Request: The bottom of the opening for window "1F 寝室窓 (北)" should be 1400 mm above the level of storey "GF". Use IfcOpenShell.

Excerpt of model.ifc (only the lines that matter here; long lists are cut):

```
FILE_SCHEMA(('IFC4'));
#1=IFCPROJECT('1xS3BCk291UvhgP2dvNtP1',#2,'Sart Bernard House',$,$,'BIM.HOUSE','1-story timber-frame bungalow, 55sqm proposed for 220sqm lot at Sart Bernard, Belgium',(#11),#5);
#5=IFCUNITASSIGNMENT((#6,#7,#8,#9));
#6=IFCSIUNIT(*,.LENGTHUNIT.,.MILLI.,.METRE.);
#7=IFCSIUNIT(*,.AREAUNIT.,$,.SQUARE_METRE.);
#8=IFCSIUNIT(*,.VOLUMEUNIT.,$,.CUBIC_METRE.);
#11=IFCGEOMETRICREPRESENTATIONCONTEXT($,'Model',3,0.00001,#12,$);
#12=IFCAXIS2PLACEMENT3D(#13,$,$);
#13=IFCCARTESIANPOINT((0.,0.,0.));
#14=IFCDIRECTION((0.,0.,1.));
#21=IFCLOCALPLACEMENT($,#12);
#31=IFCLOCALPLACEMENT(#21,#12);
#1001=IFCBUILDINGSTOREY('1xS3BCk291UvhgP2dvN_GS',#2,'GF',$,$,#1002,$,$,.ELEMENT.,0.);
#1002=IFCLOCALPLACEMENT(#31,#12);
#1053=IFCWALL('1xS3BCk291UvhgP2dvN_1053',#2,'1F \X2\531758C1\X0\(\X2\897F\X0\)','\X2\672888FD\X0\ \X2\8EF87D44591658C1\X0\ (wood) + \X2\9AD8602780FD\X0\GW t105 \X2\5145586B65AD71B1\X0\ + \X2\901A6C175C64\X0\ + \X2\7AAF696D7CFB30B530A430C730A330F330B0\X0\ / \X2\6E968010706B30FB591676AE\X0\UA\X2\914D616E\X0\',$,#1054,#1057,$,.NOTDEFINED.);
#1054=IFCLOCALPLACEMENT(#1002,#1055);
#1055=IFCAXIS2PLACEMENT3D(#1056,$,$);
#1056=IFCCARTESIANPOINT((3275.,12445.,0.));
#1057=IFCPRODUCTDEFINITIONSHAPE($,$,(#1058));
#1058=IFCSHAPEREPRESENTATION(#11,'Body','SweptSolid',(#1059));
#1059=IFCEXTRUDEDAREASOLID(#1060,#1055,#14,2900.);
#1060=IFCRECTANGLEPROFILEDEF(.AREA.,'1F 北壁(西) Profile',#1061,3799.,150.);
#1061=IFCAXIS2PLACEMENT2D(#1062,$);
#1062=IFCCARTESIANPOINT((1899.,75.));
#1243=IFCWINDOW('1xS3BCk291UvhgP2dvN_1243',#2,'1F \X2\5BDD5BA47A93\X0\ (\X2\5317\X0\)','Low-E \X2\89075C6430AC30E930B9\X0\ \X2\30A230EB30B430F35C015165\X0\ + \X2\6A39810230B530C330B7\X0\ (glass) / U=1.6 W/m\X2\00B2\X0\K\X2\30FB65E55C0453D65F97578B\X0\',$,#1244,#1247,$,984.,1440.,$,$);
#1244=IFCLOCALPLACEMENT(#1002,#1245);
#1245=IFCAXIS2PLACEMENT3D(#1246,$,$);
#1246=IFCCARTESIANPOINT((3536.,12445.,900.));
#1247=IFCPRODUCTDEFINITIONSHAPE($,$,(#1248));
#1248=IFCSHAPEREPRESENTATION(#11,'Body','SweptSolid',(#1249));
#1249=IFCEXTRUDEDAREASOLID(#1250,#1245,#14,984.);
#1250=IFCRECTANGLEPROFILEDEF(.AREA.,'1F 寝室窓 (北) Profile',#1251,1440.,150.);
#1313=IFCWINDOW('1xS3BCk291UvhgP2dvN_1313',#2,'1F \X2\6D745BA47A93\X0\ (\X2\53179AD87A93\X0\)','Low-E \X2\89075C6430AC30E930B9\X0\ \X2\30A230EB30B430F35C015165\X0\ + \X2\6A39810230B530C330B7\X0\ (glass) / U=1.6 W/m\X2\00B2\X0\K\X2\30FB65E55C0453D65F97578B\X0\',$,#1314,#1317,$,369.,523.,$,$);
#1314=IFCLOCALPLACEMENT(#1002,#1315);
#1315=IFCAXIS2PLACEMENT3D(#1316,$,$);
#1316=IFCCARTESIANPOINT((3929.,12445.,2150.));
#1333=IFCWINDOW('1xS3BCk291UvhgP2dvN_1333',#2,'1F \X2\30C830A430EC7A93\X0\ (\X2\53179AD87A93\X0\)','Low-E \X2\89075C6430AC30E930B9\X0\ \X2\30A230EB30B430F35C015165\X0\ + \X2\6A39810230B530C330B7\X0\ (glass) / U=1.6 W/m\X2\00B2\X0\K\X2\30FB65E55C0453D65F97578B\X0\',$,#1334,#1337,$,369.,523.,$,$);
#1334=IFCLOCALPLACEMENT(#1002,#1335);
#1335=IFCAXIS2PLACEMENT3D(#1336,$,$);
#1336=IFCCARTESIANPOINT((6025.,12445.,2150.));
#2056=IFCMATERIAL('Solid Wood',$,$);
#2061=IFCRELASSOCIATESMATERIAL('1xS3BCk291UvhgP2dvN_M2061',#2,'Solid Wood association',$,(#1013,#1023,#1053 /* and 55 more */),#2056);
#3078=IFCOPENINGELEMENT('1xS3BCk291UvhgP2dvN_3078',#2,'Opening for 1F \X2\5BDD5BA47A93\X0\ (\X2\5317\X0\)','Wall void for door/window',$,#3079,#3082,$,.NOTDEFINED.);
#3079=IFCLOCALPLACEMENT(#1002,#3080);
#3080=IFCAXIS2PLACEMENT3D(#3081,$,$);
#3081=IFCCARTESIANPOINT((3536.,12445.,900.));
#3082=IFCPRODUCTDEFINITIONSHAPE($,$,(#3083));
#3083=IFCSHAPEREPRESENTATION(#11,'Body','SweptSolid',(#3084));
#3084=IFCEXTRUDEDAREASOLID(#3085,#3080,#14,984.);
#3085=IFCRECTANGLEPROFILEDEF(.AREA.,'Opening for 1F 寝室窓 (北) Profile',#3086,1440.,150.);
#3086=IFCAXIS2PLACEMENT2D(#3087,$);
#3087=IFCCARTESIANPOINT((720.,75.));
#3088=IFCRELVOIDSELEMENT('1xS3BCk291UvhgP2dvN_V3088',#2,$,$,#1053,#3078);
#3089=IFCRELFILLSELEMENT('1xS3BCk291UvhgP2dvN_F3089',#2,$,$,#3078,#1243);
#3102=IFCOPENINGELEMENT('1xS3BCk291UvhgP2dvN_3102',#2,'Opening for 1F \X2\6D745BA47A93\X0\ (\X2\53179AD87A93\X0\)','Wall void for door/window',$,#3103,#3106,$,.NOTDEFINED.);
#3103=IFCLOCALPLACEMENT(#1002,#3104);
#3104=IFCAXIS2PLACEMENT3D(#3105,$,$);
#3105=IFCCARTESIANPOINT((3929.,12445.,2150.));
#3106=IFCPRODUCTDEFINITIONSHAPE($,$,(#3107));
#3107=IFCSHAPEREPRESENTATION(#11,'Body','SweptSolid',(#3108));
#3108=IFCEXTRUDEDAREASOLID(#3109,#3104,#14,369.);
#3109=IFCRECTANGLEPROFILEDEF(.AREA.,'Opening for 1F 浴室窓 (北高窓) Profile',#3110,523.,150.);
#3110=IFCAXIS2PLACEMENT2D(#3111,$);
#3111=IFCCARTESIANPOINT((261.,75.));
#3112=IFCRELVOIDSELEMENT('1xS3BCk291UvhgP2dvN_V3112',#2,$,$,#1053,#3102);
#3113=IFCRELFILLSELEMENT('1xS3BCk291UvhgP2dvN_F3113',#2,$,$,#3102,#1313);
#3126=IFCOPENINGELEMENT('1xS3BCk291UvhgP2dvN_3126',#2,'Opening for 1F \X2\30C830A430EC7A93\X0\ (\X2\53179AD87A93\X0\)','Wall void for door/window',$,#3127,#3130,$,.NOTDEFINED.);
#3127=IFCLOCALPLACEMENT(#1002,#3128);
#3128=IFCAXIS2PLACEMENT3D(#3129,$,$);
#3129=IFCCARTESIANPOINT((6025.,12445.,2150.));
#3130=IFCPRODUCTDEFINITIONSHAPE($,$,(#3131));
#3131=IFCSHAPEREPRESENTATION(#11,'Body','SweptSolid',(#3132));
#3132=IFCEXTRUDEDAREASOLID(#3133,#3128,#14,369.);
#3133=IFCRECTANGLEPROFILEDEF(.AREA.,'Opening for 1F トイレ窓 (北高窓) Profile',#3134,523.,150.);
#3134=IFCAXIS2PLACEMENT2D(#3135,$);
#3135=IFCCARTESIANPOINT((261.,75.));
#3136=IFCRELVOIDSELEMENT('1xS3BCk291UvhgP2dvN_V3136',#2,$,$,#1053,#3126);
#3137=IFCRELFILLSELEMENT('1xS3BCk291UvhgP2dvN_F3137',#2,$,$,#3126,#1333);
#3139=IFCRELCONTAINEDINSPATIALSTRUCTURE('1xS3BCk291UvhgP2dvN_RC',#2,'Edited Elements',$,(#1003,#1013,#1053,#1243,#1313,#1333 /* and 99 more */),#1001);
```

```python
import numpy as np
import ifcopenshell
import ifcopenshell.api.geometry
import ifcopenshell.geom
import ifcopenshell.util.element
import ifcopenshell.util.placement
import ifcopenshell.util.shape
import ifcopenshell.util.unit

model = ifcopenshell.open("model.ifc")
unit_scale = ifcopenshell.util.unit.calculate_unit_scale(model)

window = model.by_guid("1xS3BCk291UvhgP2dvN_1243")
opening = window.FillsVoids[0].RelatingOpeningElement
storey = ifcopenshell.util.element.get_container(window, ifc_class="IfcBuildingStorey")
level = ifcopenshell.util.placement.get_local_placement(storey.ObjectPlacement)[2, 3]

# The opening's origin need not be at the sill, so measure its lowest point.
shape = ifcopenshell.geom.create_shape(ifcopenshell.geom.settings(), opening)
bottom = ifcopenshell.util.shape.get_shape_bottom_elevation(shape, shape.geometry) / unit_scale
dz = level + 1400.0 - bottom

shift = np.array([0.0, 0.0, dz])
# The window is not placed relative to its opening, so move both.
for product in (opening, window):
    matrix = ifcopenshell.util.placement.get_local_placement(product.ObjectPlacement)
    matrix[:3, 3] += shift
    ifcopenshell.api.geometry.edit_object_placement(model, product=product, matrix=matrix, is_si=False)

print(f"moved by {dz * unit_scale:+.3f} m")

model.write("model_v2.ifc")
```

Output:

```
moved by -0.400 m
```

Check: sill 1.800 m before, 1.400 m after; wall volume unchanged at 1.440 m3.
